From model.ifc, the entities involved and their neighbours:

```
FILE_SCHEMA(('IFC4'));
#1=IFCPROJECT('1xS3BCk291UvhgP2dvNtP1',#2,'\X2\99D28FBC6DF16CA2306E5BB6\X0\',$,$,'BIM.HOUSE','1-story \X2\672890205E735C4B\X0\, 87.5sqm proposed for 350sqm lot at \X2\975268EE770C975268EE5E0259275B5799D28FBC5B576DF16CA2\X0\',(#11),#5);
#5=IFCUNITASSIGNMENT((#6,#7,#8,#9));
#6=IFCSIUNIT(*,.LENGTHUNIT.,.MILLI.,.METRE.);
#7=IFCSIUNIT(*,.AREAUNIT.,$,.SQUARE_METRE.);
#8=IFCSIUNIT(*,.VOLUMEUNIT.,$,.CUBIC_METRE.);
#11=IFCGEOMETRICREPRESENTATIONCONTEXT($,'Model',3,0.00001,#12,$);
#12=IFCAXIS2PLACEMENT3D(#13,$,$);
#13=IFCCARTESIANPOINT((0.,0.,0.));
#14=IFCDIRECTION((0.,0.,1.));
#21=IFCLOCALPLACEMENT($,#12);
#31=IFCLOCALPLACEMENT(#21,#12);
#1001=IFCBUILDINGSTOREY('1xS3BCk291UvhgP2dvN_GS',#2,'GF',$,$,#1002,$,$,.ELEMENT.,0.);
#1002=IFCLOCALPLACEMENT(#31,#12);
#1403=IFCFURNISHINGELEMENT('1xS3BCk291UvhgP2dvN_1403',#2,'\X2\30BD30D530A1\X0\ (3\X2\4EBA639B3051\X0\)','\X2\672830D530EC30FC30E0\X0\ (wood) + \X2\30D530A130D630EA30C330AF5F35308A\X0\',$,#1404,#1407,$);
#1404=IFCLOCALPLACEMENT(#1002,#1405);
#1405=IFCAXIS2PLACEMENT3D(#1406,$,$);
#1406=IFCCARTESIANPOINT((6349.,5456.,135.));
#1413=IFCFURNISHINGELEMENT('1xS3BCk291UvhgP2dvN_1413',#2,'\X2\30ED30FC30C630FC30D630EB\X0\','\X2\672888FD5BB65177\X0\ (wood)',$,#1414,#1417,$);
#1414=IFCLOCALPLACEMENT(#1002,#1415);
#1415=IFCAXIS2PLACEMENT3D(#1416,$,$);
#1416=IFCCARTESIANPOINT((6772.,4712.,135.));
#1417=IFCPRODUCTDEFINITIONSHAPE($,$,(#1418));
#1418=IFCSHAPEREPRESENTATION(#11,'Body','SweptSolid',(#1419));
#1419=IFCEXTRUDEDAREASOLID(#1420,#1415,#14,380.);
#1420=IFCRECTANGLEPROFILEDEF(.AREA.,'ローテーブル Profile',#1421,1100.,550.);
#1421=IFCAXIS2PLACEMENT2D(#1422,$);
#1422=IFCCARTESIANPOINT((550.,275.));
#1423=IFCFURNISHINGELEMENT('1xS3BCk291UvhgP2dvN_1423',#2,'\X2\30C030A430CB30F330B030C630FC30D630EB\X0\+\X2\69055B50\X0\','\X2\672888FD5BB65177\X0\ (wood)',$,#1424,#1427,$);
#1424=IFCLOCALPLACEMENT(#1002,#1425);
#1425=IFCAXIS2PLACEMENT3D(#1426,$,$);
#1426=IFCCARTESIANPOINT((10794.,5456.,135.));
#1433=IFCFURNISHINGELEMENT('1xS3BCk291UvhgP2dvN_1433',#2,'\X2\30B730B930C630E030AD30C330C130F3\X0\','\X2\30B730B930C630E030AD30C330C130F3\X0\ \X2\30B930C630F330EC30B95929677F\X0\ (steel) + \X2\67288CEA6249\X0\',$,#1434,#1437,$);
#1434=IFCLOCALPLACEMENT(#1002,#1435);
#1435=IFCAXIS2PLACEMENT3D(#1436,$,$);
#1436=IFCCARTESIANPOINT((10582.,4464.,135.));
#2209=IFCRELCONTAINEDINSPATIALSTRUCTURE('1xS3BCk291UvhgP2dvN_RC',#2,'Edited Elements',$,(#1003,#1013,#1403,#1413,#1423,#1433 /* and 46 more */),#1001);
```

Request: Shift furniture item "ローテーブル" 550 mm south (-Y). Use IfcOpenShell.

```python
import ifcopenshell
import ifcopenshell.api.geometry
import ifcopenshell.util.placement
import ifcopenshell.util.unit

model = ifcopenshell.open("model.ifc")
unit_scale = ifcopenshell.util.unit.calculate_unit_scale(model)

item = model.by_id(1413)
matrix = ifcopenshell.util.placement.get_local_placement(item.ObjectPlacement)
matrix[1, 3] -= 0.55 / unit_scale
ifcopenshell.api.geometry.edit_object_placement(model, product=item, matrix=matrix, is_si=False)

print(ifcopenshell.util.placement.get_local_placement(item.ObjectPlacement).round(3) + 0.0)

model.write("model_updated.ifc")
```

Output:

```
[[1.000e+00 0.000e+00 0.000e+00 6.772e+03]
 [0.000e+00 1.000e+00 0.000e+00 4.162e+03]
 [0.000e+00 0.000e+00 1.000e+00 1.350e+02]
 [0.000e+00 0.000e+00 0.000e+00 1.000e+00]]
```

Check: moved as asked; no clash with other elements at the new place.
